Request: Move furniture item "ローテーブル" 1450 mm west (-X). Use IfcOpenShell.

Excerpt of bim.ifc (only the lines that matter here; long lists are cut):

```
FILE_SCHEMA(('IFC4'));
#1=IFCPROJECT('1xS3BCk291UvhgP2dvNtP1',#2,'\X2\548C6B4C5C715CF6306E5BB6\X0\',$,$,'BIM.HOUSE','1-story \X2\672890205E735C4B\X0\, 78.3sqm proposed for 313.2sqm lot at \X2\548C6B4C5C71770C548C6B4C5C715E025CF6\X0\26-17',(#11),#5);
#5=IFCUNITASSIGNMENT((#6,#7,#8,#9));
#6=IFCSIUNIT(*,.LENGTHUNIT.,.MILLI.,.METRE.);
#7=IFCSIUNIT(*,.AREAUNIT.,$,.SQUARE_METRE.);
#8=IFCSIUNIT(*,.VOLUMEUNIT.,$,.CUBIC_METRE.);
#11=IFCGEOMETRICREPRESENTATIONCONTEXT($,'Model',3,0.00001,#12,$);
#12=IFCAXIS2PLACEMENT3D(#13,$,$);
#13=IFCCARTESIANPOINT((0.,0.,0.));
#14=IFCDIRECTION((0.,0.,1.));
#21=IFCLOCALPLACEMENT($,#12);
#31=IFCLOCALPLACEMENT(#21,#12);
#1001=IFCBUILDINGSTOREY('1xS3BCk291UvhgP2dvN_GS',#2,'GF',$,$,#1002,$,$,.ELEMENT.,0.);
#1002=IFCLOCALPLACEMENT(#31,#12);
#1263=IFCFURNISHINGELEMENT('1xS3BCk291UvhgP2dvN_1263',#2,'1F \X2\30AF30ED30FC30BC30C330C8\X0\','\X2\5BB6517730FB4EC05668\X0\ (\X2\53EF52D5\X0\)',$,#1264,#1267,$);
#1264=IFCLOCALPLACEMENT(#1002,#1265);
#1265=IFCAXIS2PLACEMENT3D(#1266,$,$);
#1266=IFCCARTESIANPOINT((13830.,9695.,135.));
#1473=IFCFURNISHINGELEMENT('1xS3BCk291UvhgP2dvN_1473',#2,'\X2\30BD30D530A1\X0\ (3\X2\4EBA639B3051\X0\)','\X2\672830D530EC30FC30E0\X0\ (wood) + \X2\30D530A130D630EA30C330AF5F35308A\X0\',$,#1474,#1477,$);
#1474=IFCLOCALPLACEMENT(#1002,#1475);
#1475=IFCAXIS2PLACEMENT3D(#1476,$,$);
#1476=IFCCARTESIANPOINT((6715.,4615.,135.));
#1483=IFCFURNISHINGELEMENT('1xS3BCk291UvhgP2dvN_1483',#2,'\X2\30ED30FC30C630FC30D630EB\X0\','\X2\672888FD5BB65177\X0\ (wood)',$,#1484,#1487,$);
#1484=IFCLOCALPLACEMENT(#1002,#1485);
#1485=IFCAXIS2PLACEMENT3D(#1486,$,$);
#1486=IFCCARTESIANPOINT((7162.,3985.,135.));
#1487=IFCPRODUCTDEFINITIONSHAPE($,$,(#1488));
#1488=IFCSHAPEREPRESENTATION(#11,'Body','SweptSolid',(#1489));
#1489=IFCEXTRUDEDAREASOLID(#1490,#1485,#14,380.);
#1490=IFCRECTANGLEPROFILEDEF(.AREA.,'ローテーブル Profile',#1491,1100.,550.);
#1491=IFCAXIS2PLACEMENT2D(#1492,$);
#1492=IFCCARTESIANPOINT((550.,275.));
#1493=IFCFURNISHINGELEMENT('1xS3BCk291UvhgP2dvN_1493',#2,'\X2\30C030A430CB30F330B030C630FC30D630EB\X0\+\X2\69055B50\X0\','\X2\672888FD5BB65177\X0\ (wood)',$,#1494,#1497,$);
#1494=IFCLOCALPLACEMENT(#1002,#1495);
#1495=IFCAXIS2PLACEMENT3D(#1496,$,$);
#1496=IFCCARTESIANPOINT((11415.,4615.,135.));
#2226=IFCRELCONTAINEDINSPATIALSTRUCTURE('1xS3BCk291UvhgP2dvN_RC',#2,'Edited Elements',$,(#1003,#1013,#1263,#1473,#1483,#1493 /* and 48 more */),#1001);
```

```python
import ifcopenshell
import ifcopenshell.api.geometry
import ifcopenshell.util.placement
import ifcopenshell.util.unit

model = ifcopenshell.open("bim.ifc")
unit_scale = ifcopenshell.util.unit.calculate_unit_scale(model)

item = model.by_id(1483)
matrix = ifcopenshell.util.placement.get_local_placement(item.ObjectPlacement)
matrix[0, 3] -= 1.45 / unit_scale
ifcopenshell.api.geometry.edit_object_placement(model, product=item, matrix=matrix, is_si=False)

print(ifcopenshell.util.placement.get_local_placement(item.ObjectPlacement).round(3) + 0.0)

model.write("bim_edited.ifc")
```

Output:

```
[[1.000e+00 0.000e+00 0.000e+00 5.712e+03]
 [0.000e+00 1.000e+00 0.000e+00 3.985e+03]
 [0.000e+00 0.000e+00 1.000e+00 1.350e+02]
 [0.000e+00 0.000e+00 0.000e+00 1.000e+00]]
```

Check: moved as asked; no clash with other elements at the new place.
